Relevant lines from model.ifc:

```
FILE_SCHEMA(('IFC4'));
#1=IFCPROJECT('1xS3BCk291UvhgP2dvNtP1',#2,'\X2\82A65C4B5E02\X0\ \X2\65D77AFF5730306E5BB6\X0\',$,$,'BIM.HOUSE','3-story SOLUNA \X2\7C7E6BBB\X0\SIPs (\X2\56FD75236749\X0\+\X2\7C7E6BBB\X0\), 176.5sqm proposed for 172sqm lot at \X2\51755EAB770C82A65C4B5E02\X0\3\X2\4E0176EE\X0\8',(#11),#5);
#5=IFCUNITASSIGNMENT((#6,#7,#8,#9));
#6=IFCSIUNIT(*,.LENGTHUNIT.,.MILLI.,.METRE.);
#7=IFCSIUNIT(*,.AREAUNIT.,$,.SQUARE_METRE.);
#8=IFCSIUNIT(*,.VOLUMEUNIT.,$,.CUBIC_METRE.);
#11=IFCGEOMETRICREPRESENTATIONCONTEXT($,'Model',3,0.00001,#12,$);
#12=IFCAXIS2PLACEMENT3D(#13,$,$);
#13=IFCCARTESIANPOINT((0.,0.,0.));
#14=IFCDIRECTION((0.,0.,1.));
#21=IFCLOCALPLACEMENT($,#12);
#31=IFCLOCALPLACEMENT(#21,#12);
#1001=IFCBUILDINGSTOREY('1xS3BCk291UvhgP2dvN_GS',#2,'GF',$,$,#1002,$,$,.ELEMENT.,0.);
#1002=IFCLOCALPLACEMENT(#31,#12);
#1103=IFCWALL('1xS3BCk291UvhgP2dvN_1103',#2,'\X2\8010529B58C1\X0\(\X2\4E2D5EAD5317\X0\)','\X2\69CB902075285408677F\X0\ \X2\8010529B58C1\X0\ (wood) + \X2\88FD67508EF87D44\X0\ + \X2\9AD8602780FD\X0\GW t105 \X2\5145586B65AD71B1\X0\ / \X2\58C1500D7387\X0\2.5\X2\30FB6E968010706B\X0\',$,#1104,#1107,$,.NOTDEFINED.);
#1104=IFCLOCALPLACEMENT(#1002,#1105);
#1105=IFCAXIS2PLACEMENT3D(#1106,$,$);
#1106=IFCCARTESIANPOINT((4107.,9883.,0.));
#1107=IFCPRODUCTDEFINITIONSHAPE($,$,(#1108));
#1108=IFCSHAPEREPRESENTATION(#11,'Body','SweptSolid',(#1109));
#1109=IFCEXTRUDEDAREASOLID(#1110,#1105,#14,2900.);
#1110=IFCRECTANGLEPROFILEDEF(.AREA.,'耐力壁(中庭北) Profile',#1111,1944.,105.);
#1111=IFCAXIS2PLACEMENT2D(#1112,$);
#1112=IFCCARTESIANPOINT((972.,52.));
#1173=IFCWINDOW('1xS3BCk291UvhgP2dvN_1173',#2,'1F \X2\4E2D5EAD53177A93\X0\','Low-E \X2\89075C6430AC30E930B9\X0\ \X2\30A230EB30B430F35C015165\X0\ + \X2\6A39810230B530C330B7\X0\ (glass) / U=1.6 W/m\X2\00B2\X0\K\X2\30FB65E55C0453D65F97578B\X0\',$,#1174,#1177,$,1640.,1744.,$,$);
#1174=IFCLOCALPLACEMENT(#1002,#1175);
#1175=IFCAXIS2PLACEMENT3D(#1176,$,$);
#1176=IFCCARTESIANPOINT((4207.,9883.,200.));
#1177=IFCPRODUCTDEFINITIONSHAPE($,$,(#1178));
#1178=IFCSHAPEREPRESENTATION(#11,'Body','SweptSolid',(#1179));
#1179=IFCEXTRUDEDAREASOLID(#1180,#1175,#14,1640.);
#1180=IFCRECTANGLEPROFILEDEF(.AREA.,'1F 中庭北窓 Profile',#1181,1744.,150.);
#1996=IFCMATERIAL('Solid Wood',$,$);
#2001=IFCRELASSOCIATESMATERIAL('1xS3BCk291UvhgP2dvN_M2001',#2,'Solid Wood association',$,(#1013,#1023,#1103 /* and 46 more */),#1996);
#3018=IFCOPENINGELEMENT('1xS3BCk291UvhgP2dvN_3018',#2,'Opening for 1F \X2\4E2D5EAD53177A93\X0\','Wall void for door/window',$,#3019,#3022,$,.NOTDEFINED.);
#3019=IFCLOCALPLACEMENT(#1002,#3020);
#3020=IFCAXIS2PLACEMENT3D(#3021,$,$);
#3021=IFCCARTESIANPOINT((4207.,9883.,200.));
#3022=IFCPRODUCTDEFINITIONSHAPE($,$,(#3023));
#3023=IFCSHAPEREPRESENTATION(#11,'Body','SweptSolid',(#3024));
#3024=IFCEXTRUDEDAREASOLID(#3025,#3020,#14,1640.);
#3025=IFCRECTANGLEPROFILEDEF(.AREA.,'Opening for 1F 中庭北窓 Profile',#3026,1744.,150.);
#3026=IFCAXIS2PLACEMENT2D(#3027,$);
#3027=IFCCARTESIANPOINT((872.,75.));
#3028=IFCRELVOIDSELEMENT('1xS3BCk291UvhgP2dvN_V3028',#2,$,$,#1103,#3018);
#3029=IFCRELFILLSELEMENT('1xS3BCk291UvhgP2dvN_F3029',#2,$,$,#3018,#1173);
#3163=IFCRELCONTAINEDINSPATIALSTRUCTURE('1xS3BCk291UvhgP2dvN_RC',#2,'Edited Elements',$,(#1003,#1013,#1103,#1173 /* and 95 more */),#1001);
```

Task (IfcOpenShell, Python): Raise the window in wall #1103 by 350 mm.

```python
import numpy as np
import ifcopenshell
import ifcopenshell.api.geometry
import ifcopenshell.util.placement
import ifcopenshell.util.unit

model = ifcopenshell.open("model.ifc")
unit_scale = ifcopenshell.util.unit.calculate_unit_scale(model)

window = model.by_id(1173)
opening = window.FillsVoids[0].RelatingOpeningElement
dz = 0.35 / unit_scale

shift = np.array([0.0, 0.0, dz])
# The window is not placed relative to its opening, so move both.
for product in (opening, window):
    matrix = ifcopenshell.util.placement.get_local_placement(product.ObjectPlacement)
    matrix[:3, 3] += shift
    ifcopenshell.api.geometry.edit_object_placement(model, product=product, matrix=matrix, is_si=False)

print(f"moved by {dz * unit_scale:+.3f} m")

model.write("model_rev.ifc")
```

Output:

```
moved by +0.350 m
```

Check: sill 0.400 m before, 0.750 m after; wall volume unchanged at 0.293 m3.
